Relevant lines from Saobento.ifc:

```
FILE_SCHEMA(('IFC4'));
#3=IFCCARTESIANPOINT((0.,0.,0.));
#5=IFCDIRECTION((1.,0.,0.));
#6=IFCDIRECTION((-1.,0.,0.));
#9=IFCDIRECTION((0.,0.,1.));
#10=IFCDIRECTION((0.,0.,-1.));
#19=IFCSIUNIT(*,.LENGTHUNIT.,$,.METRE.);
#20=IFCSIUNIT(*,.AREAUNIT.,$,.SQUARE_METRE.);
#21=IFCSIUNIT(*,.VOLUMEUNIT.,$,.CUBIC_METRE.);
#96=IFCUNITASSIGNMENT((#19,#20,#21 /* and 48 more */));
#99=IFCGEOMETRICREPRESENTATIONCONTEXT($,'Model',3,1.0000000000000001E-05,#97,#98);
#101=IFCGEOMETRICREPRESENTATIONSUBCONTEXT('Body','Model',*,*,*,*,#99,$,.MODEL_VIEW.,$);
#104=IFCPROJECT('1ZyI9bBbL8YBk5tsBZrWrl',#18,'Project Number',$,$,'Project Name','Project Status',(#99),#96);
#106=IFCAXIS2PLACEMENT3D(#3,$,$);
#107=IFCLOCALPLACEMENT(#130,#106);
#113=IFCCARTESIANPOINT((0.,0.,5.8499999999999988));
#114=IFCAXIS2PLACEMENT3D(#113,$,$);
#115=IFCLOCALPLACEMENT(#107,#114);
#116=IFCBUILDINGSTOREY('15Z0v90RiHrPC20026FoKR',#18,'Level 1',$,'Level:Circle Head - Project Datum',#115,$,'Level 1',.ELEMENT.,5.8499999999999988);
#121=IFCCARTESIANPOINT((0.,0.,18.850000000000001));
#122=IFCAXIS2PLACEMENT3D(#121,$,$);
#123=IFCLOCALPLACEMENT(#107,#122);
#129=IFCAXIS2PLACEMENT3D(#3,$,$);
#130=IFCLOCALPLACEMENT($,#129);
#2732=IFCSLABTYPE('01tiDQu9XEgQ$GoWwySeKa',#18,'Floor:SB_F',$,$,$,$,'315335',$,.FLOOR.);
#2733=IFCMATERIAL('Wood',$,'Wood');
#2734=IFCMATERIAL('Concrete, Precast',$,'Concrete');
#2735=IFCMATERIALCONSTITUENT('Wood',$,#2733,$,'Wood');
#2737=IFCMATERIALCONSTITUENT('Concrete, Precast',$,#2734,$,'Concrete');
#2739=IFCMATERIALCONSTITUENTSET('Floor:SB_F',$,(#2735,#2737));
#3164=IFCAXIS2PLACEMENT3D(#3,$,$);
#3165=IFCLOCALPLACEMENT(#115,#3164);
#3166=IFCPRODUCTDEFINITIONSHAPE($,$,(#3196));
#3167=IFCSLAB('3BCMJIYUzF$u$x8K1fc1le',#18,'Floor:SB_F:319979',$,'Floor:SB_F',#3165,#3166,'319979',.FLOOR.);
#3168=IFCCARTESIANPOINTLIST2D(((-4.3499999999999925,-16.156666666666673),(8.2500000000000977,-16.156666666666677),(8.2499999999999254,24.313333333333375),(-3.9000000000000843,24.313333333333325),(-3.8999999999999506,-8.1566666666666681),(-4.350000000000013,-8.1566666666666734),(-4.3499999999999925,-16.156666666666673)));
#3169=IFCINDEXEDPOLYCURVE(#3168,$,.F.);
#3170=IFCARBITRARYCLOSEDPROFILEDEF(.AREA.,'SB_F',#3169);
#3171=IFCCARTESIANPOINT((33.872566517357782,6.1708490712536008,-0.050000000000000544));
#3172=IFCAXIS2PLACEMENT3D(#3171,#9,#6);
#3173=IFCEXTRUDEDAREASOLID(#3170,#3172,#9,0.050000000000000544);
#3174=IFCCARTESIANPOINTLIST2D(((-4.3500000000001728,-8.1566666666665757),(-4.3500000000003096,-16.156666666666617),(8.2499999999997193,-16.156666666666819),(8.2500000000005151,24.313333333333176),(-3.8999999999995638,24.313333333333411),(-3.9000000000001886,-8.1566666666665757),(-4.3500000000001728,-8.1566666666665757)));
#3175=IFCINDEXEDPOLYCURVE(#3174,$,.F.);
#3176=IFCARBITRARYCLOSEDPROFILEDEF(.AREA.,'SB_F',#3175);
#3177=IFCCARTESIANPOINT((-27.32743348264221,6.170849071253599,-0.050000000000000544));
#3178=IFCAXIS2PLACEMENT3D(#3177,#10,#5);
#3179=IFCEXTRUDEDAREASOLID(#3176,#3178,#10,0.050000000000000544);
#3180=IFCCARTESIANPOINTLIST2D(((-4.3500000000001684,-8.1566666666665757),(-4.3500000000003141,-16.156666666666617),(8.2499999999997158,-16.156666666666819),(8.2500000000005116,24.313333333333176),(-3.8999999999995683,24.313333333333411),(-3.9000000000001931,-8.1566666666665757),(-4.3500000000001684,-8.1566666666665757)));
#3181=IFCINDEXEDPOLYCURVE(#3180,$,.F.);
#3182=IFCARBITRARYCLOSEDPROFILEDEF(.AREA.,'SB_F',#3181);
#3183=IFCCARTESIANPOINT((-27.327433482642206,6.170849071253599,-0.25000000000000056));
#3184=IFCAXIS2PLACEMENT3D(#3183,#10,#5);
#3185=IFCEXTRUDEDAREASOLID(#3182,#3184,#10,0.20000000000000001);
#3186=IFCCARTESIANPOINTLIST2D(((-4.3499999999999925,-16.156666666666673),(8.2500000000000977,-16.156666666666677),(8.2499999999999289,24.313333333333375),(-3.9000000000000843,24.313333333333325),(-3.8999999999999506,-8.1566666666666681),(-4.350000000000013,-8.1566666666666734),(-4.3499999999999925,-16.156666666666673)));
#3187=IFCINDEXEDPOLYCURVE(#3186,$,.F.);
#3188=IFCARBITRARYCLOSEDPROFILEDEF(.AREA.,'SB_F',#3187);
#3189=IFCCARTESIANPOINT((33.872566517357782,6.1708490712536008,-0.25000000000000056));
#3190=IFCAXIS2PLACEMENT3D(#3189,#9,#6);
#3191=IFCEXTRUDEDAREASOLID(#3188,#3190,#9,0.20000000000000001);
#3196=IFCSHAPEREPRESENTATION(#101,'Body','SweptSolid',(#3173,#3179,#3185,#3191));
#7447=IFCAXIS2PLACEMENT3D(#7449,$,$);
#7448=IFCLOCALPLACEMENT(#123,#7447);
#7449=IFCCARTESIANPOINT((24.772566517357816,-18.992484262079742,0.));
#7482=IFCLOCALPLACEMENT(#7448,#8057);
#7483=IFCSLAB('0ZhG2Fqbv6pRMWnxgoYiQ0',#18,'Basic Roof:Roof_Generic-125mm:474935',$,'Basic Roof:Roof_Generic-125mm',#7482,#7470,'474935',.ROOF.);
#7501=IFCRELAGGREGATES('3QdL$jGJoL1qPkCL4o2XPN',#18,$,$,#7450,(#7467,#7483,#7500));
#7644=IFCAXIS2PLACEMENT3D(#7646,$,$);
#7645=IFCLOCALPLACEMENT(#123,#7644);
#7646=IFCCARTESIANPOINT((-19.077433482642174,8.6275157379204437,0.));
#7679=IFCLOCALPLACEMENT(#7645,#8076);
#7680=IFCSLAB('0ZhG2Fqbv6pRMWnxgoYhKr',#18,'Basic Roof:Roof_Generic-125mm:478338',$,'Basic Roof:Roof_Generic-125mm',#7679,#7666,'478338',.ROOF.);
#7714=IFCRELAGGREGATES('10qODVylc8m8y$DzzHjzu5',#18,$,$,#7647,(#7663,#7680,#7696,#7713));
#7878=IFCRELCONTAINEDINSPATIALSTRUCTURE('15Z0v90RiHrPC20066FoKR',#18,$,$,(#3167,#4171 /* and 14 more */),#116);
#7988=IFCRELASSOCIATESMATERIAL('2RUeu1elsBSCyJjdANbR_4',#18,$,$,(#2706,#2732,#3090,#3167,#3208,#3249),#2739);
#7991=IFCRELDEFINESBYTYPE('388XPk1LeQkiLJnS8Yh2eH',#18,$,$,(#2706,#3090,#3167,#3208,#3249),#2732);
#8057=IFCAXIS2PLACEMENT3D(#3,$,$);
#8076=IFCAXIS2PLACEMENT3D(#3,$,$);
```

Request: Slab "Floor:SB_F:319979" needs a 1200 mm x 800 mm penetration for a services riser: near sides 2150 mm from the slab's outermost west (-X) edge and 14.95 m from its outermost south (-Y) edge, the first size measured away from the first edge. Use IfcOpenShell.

```python
import numpy as np
import ifcopenshell
import ifcopenshell.api.feature
import ifcopenshell.api.geometry
import ifcopenshell.api.root
import ifcopenshell.geom
import ifcopenshell.util.placement
import ifcopenshell.util.representation
import ifcopenshell.util.shape
import ifcopenshell.util.unit

model = ifcopenshell.open("Saobento.ifc")
unit_scale = ifcopenshell.util.unit.calculate_unit_scale(model)
settings = ifcopenshell.geom.settings()


def volume(element):
    """Net volume in cubic metres, openings subtracted."""
    shape = ifcopenshell.geom.create_shape(settings, element)
    return ifcopenshell.util.shape.get_volume(shape.geometry)


slab = model.by_guid("3BCMJIYUzF$u$x8K1fc1le")
before = volume(slab)

# Extent in the slab's own axes, in metres. The edges named are its -X and -Y sides.
slab_shape = ifcopenshell.geom.create_shape(settings, slab)
vertices = ifcopenshell.util.shape.get_vertices(slab_shape.geometry)
x_min, y_min, bottom = vertices.min(axis=0)
top = vertices[:, 2].max()

opening = ifcopenshell.api.root.create_entity(model, ifc_class="IfcOpeningElement", name="Services riser opening", predefined_type="OPENING")
context = ifcopenshell.util.representation.get_context(model, "Model", "Body", "MODEL_VIEW")
width, depth = 1.2, 0.8
outline = [(0.0, 0.0), (width, 0.0), (width, depth), (0.0, depth), (0.0, 0.0)]
# Overshoot both faces by 50 mm so the cut is clean.
shape = ifcopenshell.api.geometry.add_slab_representation(
    model, context=context, depth=top - bottom + 0.1, polyline=outline
)
ifcopenshell.api.geometry.assign_representation(model, product=opening, representation=shape)

matrix = ifcopenshell.util.placement.get_local_placement(slab.ObjectPlacement)
matrix[:, 3] = matrix @ np.append(np.array([x_min + 2.15, y_min + 14.95, bottom - 0.05]) / unit_scale, 1.0)
ifcopenshell.api.geometry.edit_object_placement(model, product=opening, matrix=matrix, is_si=False)
ifcopenshell.api.feature.add_feature(model, feature=opening, element=slab)

after = volume(slab)

print(f"slab volume {before:.3f} -> {after:.3f} m3")

model.write("Saobento-out.ifc")
```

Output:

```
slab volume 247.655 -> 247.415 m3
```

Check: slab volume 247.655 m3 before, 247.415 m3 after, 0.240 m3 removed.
